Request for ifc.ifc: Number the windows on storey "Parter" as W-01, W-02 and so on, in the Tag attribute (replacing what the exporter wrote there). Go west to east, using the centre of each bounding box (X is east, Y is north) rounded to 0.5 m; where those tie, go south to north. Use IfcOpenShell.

First a look at what the model holds.

```python
import ifcopenshell
import ifcopenshell.util.element
import ifcopenshell.util.placement

model = ifcopenshell.open("ifc.ifc")
print(model.schema)
storey = next(s for s in model.by_type("IfcBuildingStorey") if s.Name == "Parter")
windows = [e for e in ifcopenshell.util.element.get_decomposition(storey) if e.is_a("IfcWindow")]
for e in sorted(windows, key=lambda e: e.id()):
    origin = ifcopenshell.util.placement.get_local_placement(e.ObjectPlacement)[:3, 3]
    print(e.id(), e.Tag, e.Name, origin.round(2) + 0.0, sep=" | ")
```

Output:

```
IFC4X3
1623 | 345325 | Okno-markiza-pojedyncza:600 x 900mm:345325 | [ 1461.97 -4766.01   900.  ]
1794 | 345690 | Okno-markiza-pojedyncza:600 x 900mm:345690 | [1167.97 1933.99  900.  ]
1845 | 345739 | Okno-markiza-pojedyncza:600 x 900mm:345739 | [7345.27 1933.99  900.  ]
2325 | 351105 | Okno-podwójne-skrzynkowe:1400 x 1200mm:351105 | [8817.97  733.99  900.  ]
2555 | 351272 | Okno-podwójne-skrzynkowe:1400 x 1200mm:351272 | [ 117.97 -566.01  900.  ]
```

```python
import ifcopenshell
import ifcopenshell.geom
import ifcopenshell.util.element
import ifcopenshell.util.shape

model = ifcopenshell.open("ifc.ifc")
settings = ifcopenshell.geom.settings()
settings.set("use-world-coords", True)


def centre(element):
    shape = ifcopenshell.geom.create_shape(settings, element)
    return ifcopenshell.util.shape.get_bbox_centroid(shape.geometry)


storey = next(s for s in model.by_type("IfcBuildingStorey") if s.Name == "Parter")
windows = [e for e in ifcopenshell.util.element.get_decomposition(storey) if e.is_a("IfcWindow")]

# Insertion points can sit at a corner or the storey origin, so sort by the geometry (in metres).
centres = {e: centre(e) for e in windows}
windows.sort(key=lambda e: (round(centres[e][0] / 0.5), centres[e][1]))

for i, e in enumerate(windows, start=1):
    number = f"W-{i:02d}"
    e.Tag = number
    print(e.id(), number)

model.write("ifc_updated.ifc")
```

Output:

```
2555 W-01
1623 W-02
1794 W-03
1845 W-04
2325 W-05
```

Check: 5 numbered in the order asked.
